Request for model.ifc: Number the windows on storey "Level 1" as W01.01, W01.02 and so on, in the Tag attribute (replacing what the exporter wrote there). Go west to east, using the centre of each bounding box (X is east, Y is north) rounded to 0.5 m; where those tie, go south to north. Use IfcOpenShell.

First a look at what the model holds.

```python
import ifcopenshell
import ifcopenshell.util.element
import ifcopenshell.util.placement

model = ifcopenshell.open("model.ifc")
print(model.schema)
storey = next(s for s in model.by_type("IfcBuildingStorey") if s.Name == "Level 1")
windows = [e for e in ifcopenshell.util.element.get_decomposition(storey) if e.is_a("IfcWindow")]
for e in sorted(windows, key=lambda e: e.id()):
    origin = ifcopenshell.util.placement.get_local_placement(e.ObjectPlacement)[:3, 3]
    print(e.id(), e.Tag, e.Name, origin.round(2) + 0.0, sep=" | ")
```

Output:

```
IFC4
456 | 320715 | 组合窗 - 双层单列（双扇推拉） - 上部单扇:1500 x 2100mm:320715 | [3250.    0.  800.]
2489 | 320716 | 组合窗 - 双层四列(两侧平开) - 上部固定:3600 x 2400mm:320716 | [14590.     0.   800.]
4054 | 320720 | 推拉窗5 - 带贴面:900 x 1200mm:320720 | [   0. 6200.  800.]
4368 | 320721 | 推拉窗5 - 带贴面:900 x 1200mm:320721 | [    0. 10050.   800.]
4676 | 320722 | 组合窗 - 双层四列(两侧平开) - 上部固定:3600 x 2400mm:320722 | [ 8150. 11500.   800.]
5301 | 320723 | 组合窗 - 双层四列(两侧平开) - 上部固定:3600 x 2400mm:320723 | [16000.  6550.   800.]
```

```python
import ifcopenshell
import ifcopenshell.geom
import ifcopenshell.util.element
import ifcopenshell.util.shape

model = ifcopenshell.open("model.ifc")
settings = ifcopenshell.geom.settings()
settings.set("use-world-coords", True)


def centre(element):
    shape = ifcopenshell.geom.create_shape(settings, element)
    return ifcopenshell.util.shape.get_bbox_centroid(shape.geometry)


storey = next(s for s in model.by_type("IfcBuildingStorey") if s.Name == "Level 1")
windows = [e for e in ifcopenshell.util.element.get_decomposition(storey) if e.is_a("IfcWindow")]

# Insertion points can sit at a corner or the storey origin, so sort by the geometry (in metres).
centres = {e: centre(e) for e in windows}
windows.sort(key=lambda e: (round(centres[e][0] / 0.5), centres[e][1]))

for i, e in enumerate(windows, start=1):
    number = f"W01.{i:02d}"
    e.Tag = number
    print(e.id(), number)

model.write("model_edited.ifc")
```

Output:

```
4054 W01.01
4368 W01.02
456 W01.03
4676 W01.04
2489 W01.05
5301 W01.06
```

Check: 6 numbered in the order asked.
